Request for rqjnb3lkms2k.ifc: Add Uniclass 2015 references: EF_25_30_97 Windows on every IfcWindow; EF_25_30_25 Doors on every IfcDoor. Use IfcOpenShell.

First a look at what the model holds.

```python
import ifcopenshell

model = ifcopenshell.open("rqjnb3lkms2k.ifc")
print(model.schema)
print("classifications:", [c.Name for c in model.by_type("IfcClassification")])
for ifc_class in ("IfcDoor", "IfcRoof", "IfcStair", "IfcWall", "IfcWindow"):
    print(ifc_class, len(model.by_type(ifc_class)))
```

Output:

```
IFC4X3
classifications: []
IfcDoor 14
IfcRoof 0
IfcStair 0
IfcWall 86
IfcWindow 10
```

```python
import ifcopenshell
import ifcopenshell.api.classification

model = ifcopenshell.open("rqjnb3lkms2k.ifc")

system = ifcopenshell.api.classification.add_classification(model, classification="Uniclass 2015")

codes = {
    "IfcWindow": ("EF_25_30_97", "Windows"),
    "IfcDoor": ("EF_25_30_25", "Doors"),
}
for ifc_class, (code, name) in codes.items():
    products = model.by_type(ifc_class)
    ifcopenshell.api.classification.add_reference(
        model, products=products, classification=system, identification=code, name=name
    )
    print(code, len(products))

model.write("rqjnb3lkms2k_updated.ifc")
```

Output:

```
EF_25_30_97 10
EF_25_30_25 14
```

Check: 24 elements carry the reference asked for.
